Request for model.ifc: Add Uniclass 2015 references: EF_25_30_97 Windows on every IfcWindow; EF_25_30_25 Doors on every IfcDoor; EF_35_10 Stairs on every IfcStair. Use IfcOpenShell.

First a look at what the model holds.

```python
import ifcopenshell

model = ifcopenshell.open("model.ifc")
print(model.schema)
print("classifications:", [c.Name for c in model.by_type("IfcClassification")])
for ifc_class in ("IfcDoor", "IfcRoof", "IfcStair", "IfcWall", "IfcWindow"):
    print(ifc_class, len(model.by_type(ifc_class)))
```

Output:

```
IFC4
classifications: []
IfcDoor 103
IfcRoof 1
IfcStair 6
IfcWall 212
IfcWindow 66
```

```python
import ifcopenshell
import ifcopenshell.api.classification

model = ifcopenshell.open("model.ifc")

system = ifcopenshell.api.classification.add_classification(model, classification="Uniclass 2015")

codes = {
    "IfcWindow": ("EF_25_30_97", "Windows"),
    "IfcDoor": ("EF_25_30_25", "Doors"),
    "IfcStair": ("EF_35_10", "Stairs"),
}
for ifc_class, (code, name) in codes.items():
    products = model.by_type(ifc_class)
    ifcopenshell.api.classification.add_reference(
        model, products=products, classification=system, identification=code, name=name
    )
    print(code, len(products))

model.write("model_edited.ifc")
```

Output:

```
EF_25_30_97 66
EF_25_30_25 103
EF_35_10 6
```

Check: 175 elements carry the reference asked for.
